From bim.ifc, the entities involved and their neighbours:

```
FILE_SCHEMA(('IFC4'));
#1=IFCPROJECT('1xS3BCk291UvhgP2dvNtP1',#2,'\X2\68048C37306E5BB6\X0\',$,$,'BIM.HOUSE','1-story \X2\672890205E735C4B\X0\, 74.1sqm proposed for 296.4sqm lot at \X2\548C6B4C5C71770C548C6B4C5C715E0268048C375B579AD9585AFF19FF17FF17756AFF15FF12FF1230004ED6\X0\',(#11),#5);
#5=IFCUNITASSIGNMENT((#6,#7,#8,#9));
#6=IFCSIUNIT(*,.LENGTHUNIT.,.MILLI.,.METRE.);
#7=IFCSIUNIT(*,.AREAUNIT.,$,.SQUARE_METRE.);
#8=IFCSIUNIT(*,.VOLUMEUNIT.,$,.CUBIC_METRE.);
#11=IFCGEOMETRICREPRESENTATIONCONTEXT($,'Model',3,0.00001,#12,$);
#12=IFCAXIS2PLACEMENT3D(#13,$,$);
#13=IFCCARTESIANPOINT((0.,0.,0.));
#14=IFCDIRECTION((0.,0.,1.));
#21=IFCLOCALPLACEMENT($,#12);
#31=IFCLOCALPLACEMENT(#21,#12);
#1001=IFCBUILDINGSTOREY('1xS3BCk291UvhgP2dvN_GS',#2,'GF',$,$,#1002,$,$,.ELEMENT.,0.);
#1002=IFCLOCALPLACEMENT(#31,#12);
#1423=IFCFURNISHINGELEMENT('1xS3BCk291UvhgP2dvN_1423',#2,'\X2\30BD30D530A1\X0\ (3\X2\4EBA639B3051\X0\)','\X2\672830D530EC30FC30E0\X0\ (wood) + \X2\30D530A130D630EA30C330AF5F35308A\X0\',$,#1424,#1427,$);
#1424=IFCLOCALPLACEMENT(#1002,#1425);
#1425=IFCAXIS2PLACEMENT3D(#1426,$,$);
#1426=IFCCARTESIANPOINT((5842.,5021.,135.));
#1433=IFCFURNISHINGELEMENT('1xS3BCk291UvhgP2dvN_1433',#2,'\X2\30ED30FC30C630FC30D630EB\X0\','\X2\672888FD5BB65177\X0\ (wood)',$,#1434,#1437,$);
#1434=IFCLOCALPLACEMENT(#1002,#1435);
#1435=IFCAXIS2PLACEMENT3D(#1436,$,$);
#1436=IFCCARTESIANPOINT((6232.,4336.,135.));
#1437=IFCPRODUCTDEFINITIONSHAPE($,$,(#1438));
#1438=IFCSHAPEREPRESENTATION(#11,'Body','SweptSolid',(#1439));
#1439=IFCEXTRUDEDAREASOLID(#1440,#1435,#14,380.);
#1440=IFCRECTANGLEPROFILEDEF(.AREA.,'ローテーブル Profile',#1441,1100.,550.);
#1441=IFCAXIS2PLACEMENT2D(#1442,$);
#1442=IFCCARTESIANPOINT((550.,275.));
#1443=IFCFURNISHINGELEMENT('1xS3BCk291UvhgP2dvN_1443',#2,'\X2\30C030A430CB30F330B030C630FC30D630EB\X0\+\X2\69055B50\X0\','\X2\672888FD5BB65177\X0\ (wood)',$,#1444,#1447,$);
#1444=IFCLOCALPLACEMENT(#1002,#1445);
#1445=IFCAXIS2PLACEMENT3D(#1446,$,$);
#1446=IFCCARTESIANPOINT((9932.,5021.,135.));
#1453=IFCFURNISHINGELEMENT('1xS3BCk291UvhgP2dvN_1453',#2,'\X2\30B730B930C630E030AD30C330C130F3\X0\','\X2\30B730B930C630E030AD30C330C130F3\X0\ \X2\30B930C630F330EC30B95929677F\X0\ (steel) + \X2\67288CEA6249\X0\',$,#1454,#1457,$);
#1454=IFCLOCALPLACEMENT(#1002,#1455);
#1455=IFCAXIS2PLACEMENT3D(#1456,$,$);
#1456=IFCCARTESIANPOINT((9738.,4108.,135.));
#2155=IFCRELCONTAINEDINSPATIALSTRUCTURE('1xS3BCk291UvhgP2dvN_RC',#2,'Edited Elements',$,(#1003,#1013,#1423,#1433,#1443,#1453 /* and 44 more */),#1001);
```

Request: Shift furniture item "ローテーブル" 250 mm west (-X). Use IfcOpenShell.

```python
import ifcopenshell
import ifcopenshell.api.geometry
import ifcopenshell.util.placement
import ifcopenshell.util.unit

model = ifcopenshell.open("bim.ifc")
unit_scale = ifcopenshell.util.unit.calculate_unit_scale(model)

item = model.by_id(1433)
matrix = ifcopenshell.util.placement.get_local_placement(item.ObjectPlacement)
matrix[0, 3] -= 0.25 / unit_scale
ifcopenshell.api.geometry.edit_object_placement(model, product=item, matrix=matrix, is_si=False)

print(ifcopenshell.util.placement.get_local_placement(item.ObjectPlacement).round(3) + 0.0)

model.write("bim_updated.ifc")
```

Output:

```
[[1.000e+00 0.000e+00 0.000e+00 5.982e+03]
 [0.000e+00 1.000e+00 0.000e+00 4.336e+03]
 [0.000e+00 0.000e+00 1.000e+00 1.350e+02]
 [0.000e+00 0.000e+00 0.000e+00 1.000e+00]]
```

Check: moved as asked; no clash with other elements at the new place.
